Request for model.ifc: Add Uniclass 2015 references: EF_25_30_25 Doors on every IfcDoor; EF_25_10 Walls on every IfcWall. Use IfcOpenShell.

First a look at what the model holds.

```python
import ifcopenshell

model = ifcopenshell.open("model.ifc")
print(model.schema)
print("classifications:", [c.Name for c in model.by_type("IfcClassification")])
for ifc_class in ("IfcDoor", "IfcRoof", "IfcStair", "IfcWall", "IfcWindow"):
    print(ifc_class, len(model.by_type(ifc_class)))
```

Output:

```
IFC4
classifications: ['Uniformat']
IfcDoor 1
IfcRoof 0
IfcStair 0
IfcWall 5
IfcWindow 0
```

```python
import ifcopenshell
import ifcopenshell.api.classification

model = ifcopenshell.open("model.ifc")

system = ifcopenshell.api.classification.add_classification(model, classification="Uniclass 2015")

codes = {
    "IfcDoor": ("EF_25_30_25", "Doors"),
    "IfcWall": ("EF_25_10", "Walls"),
}
for ifc_class, (code, name) in codes.items():
    products = model.by_type(ifc_class)
    ifcopenshell.api.classification.add_reference(
        model, products=products, classification=system, identification=code, name=name
    )
    print(code, len(products))

model.write("model_rev.ifc")
```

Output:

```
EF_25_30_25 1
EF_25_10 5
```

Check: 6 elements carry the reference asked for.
